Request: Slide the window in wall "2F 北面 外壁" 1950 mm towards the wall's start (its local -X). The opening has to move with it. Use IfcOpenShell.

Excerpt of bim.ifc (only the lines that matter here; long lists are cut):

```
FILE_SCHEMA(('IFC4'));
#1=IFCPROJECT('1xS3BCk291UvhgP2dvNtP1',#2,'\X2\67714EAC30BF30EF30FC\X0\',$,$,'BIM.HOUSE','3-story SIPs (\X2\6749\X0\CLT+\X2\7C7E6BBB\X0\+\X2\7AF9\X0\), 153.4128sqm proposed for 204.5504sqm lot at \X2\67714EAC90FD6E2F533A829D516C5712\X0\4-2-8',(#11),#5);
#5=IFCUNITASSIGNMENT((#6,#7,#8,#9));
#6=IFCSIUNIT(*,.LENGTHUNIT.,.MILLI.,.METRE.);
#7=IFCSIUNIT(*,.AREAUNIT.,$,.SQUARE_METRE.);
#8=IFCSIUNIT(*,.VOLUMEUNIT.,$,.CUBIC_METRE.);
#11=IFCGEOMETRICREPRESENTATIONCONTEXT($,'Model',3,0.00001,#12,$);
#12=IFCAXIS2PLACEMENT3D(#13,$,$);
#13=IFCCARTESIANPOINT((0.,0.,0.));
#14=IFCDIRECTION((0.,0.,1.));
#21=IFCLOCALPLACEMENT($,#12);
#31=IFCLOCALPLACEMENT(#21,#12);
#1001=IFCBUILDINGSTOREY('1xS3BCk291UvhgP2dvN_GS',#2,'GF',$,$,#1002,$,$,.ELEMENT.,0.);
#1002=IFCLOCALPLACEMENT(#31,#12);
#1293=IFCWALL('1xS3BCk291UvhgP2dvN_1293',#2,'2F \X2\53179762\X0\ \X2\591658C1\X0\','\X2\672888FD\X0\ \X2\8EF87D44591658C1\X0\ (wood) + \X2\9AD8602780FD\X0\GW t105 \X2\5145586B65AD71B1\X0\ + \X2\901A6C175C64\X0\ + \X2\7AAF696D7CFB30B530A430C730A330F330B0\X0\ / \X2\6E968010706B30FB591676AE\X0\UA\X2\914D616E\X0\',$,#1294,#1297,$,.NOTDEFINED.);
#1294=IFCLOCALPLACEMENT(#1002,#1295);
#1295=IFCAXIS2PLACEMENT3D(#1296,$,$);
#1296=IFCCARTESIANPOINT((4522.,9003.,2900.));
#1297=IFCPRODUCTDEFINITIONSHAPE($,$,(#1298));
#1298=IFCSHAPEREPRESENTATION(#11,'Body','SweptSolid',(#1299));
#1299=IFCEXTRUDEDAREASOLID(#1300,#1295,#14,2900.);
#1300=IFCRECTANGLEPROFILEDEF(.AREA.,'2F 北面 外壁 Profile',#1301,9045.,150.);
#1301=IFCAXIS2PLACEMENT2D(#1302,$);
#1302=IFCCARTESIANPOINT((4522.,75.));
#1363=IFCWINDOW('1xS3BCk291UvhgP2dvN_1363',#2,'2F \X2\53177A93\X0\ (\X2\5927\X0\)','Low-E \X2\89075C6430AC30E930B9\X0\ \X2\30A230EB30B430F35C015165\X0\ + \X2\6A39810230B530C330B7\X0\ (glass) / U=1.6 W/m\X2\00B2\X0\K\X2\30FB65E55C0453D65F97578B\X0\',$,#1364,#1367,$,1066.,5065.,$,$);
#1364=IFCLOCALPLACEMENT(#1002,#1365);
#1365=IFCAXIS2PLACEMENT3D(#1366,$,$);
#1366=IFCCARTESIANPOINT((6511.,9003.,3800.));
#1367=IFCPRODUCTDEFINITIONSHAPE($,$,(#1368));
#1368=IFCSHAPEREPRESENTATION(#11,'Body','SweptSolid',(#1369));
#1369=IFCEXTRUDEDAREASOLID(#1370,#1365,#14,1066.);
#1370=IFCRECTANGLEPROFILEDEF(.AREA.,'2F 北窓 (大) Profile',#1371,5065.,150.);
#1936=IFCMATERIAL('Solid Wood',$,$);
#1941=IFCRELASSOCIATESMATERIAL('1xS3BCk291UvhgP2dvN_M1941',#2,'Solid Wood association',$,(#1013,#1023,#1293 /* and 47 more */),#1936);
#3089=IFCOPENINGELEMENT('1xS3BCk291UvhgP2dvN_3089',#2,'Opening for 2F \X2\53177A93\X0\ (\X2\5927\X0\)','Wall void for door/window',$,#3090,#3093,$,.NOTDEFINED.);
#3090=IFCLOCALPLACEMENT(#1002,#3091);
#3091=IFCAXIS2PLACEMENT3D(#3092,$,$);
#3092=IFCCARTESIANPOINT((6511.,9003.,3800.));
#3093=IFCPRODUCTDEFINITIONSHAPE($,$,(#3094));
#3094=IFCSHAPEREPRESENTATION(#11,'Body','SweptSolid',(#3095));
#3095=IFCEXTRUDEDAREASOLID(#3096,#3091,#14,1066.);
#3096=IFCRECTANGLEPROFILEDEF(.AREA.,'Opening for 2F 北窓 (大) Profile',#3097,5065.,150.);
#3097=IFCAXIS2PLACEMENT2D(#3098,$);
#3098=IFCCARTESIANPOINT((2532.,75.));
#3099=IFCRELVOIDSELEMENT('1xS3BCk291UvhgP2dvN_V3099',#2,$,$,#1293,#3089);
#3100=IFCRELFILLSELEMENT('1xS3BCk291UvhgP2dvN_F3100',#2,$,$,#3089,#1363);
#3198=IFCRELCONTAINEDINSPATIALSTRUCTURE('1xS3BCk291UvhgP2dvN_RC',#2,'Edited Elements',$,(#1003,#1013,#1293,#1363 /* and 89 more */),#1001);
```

```python
import ifcopenshell
import ifcopenshell.api.geometry
import ifcopenshell.util.placement
import ifcopenshell.util.unit

model = ifcopenshell.open("bim.ifc")
unit_scale = ifcopenshell.util.unit.calculate_unit_scale(model)

window = model.by_id(1363)
opening = window.FillsVoids[0].RelatingOpeningElement
wall = opening.VoidsElements[0].RelatingBuildingElement

wall_matrix = ifcopenshell.util.placement.get_local_placement(wall.ObjectPlacement)
shift = wall_matrix[:3, 0] * -1.95 / unit_scale
before = ifcopenshell.util.placement.get_local_placement(window.ObjectPlacement)[:3, 3].copy()

# The window is not placed relative to its opening, so move both.
for product in (opening, window):
    matrix = ifcopenshell.util.placement.get_local_placement(product.ObjectPlacement)
    matrix[:3, 3] += shift
    ifcopenshell.api.geometry.edit_object_placement(model, product=product, matrix=matrix, is_si=False)

after = ifcopenshell.util.placement.get_local_placement(window.ObjectPlacement)[:3, 3]
print("window moved by", (after - before).round(3) + 0.0)

model.write("bim_updated.ifc")
```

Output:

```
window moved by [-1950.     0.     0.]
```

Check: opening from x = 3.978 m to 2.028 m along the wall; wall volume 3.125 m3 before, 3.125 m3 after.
